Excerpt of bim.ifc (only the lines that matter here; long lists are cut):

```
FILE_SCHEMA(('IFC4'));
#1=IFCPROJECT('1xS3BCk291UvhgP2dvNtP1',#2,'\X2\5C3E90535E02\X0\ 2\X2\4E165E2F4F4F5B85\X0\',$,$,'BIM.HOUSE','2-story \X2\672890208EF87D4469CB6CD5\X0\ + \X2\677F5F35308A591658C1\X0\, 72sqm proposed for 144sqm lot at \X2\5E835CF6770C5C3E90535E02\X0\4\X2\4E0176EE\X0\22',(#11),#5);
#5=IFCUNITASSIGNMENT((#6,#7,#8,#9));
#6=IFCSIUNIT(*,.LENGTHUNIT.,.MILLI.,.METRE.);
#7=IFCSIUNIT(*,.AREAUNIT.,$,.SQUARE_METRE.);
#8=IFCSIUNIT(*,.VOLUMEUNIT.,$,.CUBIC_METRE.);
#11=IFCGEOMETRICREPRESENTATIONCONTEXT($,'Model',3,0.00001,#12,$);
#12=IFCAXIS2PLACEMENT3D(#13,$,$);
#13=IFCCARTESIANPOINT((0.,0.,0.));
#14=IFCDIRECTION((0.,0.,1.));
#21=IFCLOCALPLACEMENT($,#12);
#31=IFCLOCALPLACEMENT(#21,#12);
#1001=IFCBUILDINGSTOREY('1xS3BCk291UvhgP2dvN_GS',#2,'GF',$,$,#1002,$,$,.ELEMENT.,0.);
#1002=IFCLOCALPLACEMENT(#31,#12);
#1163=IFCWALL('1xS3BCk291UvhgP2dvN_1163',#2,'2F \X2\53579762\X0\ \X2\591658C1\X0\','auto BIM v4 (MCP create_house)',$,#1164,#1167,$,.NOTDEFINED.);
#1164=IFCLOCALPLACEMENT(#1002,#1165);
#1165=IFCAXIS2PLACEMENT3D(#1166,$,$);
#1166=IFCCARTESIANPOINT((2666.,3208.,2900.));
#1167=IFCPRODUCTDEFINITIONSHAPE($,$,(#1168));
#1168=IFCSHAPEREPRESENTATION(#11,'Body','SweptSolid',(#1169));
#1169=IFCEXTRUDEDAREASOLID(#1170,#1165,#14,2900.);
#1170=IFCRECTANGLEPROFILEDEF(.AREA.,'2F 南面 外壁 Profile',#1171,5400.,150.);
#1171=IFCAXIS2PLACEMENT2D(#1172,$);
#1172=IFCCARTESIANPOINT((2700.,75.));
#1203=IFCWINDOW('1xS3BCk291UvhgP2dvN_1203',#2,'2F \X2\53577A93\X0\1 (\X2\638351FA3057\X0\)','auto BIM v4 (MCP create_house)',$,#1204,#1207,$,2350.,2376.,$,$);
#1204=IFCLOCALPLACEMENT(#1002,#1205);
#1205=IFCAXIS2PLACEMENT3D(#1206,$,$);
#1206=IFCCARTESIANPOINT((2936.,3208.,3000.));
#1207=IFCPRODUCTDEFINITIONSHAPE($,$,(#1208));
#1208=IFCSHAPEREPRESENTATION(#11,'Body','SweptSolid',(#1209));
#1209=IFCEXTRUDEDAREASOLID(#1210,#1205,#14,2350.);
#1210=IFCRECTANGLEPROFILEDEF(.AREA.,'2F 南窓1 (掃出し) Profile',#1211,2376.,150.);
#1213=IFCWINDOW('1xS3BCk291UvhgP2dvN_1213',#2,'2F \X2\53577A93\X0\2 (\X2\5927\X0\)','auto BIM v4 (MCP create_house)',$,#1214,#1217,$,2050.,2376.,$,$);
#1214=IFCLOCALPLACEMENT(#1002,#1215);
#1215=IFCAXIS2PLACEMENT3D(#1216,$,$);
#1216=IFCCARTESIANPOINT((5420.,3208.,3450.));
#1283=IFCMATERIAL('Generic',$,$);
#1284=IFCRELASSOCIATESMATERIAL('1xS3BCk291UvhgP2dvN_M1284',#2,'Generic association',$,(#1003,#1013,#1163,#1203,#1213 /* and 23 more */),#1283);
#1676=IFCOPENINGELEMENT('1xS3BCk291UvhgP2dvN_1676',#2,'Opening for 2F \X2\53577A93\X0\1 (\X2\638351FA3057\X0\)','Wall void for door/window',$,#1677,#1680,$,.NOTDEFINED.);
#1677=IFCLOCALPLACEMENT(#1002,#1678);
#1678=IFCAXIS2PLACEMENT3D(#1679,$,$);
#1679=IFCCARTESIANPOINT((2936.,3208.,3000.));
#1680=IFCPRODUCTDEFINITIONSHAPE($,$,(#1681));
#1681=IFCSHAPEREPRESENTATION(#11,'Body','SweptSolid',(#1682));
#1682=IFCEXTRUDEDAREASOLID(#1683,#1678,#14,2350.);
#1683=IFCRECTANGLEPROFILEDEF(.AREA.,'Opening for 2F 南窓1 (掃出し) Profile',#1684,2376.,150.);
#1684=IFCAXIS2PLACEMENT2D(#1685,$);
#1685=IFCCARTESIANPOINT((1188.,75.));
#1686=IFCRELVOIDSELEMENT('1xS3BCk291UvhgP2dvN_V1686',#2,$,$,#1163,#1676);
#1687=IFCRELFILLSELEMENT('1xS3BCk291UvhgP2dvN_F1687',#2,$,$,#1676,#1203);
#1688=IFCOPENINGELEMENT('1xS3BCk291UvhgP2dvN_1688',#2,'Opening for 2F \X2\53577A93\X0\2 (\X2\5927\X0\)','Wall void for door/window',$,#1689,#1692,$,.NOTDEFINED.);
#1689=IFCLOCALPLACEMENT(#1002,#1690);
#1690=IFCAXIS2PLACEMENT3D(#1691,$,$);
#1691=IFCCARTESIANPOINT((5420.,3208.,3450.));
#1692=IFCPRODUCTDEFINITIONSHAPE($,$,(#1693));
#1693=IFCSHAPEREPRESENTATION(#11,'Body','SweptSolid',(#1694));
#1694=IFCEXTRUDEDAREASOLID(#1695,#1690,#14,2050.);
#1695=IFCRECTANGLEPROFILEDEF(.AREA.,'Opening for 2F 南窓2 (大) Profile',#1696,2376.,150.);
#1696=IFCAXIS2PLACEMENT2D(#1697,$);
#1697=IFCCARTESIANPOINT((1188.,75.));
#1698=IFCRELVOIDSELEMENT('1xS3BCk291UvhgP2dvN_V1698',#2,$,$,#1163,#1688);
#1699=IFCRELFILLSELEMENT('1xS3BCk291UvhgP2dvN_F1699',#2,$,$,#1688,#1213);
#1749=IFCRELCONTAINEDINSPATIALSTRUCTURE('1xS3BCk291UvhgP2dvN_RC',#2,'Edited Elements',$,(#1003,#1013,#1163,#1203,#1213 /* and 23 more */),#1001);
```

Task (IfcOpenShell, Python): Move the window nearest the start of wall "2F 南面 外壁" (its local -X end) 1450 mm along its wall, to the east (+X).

```python
import ifcopenshell
import ifcopenshell.api.geometry
import ifcopenshell.util.placement
import ifcopenshell.util.unit

model = ifcopenshell.open("bim.ifc")
unit_scale = ifcopenshell.util.unit.calculate_unit_scale(model)

window = model.by_guid("1xS3BCk291UvhgP2dvN_1203")
opening = window.FillsVoids[0].RelatingOpeningElement
wall = opening.VoidsElements[0].RelatingBuildingElement

wall_matrix = ifcopenshell.util.placement.get_local_placement(wall.ObjectPlacement)
shift = wall_matrix[:3, 0] * 1.45 / unit_scale
before = ifcopenshell.util.placement.get_local_placement(window.ObjectPlacement)[:3, 3].copy()

# The window is not placed relative to its opening, so move both.
for product in (opening, window):
    matrix = ifcopenshell.util.placement.get_local_placement(product.ObjectPlacement)
    matrix[:3, 3] += shift
    ifcopenshell.api.geometry.edit_object_placement(model, product=product, matrix=matrix, is_si=False)

after = ifcopenshell.util.placement.get_local_placement(window.ObjectPlacement)[:3, 3]
print("window moved by", (after - before).round(3) + 0.0)

model.write("bim_updated.ifc")
```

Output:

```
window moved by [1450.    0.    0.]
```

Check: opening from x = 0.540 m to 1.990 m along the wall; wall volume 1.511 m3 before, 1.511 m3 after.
